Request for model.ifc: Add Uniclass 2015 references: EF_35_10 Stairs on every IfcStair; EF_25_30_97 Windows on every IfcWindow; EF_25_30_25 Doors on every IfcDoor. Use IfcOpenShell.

First a look at what the model holds.

```python
import ifcopenshell

model = ifcopenshell.open("model.ifc")
print(model.schema)
print("classifications:", [c.Name for c in model.by_type("IfcClassification")])
for ifc_class in ("IfcDoor", "IfcRoof", "IfcStair", "IfcWall", "IfcWindow"):
    print(ifc_class, len(model.by_type(ifc_class)))
```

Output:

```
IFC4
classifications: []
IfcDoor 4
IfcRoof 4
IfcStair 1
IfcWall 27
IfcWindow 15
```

```python
import ifcopenshell
import ifcopenshell.api.classification

model = ifcopenshell.open("model.ifc")

system = ifcopenshell.api.classification.add_classification(model, classification="Uniclass 2015")

codes = {
    "IfcStair": ("EF_35_10", "Stairs"),
    "IfcWindow": ("EF_25_30_97", "Windows"),
    "IfcDoor": ("EF_25_30_25", "Doors"),
}
for ifc_class, (code, name) in codes.items():
    products = model.by_type(ifc_class)
    ifcopenshell.api.classification.add_reference(
        model, products=products, classification=system, identification=code, name=name
    )
    print(code, len(products))

model.write("model_updated.ifc")
```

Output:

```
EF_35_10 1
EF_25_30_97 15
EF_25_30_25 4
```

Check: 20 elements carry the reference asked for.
